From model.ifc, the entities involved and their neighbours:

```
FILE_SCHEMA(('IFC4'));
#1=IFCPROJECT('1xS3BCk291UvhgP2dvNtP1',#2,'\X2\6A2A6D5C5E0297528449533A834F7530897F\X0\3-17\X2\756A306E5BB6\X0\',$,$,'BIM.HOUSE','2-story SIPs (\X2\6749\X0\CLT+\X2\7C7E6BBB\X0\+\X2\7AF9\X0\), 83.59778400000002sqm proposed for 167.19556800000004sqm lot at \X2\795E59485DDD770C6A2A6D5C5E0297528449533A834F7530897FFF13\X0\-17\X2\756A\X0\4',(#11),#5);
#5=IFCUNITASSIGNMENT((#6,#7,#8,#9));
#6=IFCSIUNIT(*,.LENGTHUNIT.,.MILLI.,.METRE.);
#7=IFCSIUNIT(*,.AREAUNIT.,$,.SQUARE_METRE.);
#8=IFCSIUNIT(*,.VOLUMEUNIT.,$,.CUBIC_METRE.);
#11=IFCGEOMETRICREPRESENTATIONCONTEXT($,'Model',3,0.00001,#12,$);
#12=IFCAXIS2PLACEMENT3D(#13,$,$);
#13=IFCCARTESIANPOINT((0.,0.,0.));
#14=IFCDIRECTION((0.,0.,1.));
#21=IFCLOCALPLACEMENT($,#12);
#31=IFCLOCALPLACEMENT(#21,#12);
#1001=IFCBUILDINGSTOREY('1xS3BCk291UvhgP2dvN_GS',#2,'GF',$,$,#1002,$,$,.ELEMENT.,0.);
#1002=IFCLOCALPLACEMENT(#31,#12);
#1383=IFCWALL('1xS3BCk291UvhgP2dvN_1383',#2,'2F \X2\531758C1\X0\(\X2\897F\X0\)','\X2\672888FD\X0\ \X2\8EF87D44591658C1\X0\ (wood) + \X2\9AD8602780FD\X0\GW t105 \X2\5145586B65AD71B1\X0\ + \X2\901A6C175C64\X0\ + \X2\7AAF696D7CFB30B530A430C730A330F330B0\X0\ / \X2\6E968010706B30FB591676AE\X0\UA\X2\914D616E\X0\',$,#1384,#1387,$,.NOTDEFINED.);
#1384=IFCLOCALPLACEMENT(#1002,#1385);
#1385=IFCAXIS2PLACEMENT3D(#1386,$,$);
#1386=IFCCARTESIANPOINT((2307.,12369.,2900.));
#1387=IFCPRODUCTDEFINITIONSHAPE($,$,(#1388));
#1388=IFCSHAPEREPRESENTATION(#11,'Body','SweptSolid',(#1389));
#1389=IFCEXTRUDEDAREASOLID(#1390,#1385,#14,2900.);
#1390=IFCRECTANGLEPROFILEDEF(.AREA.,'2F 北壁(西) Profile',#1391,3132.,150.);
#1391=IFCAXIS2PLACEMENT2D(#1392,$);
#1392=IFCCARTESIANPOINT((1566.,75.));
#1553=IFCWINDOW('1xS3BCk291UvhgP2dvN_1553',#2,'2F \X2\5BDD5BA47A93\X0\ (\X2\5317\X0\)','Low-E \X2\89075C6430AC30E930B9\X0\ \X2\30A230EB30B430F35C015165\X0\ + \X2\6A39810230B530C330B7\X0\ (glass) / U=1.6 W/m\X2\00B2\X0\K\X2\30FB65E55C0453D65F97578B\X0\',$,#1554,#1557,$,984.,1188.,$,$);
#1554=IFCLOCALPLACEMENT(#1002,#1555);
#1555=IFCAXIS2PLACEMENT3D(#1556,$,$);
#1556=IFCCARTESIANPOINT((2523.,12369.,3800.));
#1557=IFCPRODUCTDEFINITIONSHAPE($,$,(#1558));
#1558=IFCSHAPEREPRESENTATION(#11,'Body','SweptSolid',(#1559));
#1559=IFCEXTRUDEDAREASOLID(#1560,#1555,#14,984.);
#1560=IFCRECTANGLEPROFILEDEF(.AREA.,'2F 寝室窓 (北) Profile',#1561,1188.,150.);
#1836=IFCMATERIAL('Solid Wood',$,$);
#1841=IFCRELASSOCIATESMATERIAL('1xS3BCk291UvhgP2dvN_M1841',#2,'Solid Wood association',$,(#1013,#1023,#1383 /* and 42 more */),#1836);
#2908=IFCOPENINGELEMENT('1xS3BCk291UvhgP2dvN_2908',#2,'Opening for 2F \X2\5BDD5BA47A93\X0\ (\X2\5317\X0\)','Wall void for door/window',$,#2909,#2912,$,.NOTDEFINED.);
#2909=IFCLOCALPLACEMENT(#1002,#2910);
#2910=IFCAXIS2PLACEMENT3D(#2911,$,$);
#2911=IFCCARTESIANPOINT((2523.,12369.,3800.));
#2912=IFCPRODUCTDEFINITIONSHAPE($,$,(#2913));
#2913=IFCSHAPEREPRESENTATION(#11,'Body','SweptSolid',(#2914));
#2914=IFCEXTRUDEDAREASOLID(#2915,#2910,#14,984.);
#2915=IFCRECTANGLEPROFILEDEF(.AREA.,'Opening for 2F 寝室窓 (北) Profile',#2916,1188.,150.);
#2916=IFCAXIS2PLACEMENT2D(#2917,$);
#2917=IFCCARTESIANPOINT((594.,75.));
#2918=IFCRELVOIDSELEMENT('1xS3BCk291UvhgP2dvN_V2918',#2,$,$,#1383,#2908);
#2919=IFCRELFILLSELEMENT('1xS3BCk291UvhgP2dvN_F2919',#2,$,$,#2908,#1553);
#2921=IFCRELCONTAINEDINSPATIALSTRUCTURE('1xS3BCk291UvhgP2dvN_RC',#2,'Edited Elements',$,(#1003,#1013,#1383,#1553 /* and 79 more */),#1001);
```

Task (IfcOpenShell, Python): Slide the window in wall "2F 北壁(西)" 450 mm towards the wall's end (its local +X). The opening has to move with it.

```python
import ifcopenshell
import ifcopenshell.api.geometry
import ifcopenshell.util.placement

model = ifcopenshell.open("model.ifc")

window = model.by_guid("1xS3BCk291UvhgP2dvN_1553")
opening = window.FillsVoids[0].RelatingOpeningElement
wall = opening.VoidsElements[0].RelatingBuildingElement

wall_matrix = ifcopenshell.util.placement.get_local_placement(wall.ObjectPlacement)
shift = wall_matrix[:3, 0] * 450.0
before = ifcopenshell.util.placement.get_local_placement(window.ObjectPlacement)[:3, 3].copy()

# The window is not placed relative to its opening, so move both.
for product in (opening, window):
    matrix = ifcopenshell.util.placement.get_local_placement(product.ObjectPlacement)
    matrix[:3, 3] += shift
    ifcopenshell.api.geometry.edit_object_placement(model, product=product, matrix=matrix, is_si=False)

after = ifcopenshell.util.placement.get_local_placement(window.ObjectPlacement)[:3, 3]
print("window moved by", (after - before).round(3) + 0.0)

model.write("model_v2.ifc")
```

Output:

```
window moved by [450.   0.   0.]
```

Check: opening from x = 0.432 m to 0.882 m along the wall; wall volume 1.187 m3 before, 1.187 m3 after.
